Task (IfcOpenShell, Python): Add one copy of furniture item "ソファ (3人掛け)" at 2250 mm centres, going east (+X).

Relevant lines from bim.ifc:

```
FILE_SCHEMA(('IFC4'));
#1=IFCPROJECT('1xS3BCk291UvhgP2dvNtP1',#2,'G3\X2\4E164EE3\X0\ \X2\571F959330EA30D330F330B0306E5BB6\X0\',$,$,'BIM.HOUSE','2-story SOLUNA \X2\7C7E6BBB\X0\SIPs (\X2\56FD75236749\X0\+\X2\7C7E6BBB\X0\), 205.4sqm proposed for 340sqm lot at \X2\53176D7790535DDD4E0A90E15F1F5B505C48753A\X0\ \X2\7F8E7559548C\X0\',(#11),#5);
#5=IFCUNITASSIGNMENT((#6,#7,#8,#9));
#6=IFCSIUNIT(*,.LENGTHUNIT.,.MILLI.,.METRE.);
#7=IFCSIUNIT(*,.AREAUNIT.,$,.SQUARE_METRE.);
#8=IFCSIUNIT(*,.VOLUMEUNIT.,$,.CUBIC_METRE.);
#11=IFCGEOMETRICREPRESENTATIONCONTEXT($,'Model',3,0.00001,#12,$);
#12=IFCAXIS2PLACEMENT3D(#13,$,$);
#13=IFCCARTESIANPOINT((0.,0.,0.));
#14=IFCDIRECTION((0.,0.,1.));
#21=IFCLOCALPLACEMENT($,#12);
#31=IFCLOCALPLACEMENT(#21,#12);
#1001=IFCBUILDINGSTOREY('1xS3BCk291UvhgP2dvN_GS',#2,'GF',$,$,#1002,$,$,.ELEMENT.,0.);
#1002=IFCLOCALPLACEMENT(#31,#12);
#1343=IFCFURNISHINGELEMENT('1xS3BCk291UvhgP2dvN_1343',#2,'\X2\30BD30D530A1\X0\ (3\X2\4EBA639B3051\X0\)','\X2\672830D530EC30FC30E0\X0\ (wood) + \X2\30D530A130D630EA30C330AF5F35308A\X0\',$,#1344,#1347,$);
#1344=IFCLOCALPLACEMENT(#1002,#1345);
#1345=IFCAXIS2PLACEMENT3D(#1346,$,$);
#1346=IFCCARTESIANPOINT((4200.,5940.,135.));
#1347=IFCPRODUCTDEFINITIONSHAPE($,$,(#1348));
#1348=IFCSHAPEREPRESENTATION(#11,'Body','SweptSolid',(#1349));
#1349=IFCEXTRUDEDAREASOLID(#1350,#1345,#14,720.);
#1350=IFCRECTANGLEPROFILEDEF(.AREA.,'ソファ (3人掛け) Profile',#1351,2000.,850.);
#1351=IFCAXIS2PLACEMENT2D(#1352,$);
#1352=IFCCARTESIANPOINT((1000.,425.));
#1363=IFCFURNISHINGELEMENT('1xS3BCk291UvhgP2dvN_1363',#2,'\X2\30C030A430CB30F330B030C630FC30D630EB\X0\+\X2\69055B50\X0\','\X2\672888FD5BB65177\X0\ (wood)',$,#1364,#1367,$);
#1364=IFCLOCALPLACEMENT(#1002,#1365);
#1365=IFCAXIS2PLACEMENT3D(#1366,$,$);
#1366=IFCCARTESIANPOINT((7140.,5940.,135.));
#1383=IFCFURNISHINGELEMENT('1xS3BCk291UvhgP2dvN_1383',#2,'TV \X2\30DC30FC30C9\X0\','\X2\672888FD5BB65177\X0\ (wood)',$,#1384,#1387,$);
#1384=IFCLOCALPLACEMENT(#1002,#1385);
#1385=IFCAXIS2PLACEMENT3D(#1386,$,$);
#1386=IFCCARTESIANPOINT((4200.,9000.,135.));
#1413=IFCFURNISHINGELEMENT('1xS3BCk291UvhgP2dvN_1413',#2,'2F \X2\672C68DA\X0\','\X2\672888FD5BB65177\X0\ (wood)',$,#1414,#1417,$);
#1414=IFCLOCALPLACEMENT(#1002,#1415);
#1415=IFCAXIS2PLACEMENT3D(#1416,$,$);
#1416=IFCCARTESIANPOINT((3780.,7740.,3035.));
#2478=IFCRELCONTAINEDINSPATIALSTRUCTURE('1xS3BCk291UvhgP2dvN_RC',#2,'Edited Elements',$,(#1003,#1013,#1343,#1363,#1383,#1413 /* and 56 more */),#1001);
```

```python
import numpy as np
import ifcopenshell
import ifcopenshell.api.geometry
import ifcopenshell.api.root
import ifcopenshell.util.element
import ifcopenshell.util.placement
import ifcopenshell.util.unit

model = ifcopenshell.open("bim.ifc")
unit_scale = ifcopenshell.util.unit.calculate_unit_scale(model)


def reuse_history(source, copy):
    """copy_class also copies each property set's owner history, people and application; keep the originals."""
    for rel in copy.IsDefinedBy:
        if rel.is_a("IfcRelDefinesByProperties") and (history := rel.RelatingPropertyDefinition.OwnerHistory):
            rel.RelatingPropertyDefinition.OwnerHistory = source.OwnerHistory
            ifcopenshell.util.element.remove_deep2(model, history)


source = model.by_guid("1xS3BCk291UvhgP2dvN_1343")
base = ifcopenshell.util.placement.get_local_placement(source.ObjectPlacement)
step = np.array([1.0, 0.0, 0.0]) * 2.25 / unit_scale

for i in range(1, 2):
    copy = ifcopenshell.api.root.copy_class(model, product=source)
    copy.Representation = ifcopenshell.util.element.copy_deep(
        model, source.Representation, exclude=["IfcGeometricRepresentationContext", "IfcRepresentationMap"]
    )
    reuse_history(source, copy)
    matrix = base.copy()
    matrix[:3, 3] += i * step
    print("added at", matrix[:3, 3].round(3) + 0.0)
    ifcopenshell.api.geometry.edit_object_placement(model, product=copy, matrix=matrix, is_si=False)

model.write("bim_updated.ifc")
```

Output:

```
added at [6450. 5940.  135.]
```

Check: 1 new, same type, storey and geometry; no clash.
